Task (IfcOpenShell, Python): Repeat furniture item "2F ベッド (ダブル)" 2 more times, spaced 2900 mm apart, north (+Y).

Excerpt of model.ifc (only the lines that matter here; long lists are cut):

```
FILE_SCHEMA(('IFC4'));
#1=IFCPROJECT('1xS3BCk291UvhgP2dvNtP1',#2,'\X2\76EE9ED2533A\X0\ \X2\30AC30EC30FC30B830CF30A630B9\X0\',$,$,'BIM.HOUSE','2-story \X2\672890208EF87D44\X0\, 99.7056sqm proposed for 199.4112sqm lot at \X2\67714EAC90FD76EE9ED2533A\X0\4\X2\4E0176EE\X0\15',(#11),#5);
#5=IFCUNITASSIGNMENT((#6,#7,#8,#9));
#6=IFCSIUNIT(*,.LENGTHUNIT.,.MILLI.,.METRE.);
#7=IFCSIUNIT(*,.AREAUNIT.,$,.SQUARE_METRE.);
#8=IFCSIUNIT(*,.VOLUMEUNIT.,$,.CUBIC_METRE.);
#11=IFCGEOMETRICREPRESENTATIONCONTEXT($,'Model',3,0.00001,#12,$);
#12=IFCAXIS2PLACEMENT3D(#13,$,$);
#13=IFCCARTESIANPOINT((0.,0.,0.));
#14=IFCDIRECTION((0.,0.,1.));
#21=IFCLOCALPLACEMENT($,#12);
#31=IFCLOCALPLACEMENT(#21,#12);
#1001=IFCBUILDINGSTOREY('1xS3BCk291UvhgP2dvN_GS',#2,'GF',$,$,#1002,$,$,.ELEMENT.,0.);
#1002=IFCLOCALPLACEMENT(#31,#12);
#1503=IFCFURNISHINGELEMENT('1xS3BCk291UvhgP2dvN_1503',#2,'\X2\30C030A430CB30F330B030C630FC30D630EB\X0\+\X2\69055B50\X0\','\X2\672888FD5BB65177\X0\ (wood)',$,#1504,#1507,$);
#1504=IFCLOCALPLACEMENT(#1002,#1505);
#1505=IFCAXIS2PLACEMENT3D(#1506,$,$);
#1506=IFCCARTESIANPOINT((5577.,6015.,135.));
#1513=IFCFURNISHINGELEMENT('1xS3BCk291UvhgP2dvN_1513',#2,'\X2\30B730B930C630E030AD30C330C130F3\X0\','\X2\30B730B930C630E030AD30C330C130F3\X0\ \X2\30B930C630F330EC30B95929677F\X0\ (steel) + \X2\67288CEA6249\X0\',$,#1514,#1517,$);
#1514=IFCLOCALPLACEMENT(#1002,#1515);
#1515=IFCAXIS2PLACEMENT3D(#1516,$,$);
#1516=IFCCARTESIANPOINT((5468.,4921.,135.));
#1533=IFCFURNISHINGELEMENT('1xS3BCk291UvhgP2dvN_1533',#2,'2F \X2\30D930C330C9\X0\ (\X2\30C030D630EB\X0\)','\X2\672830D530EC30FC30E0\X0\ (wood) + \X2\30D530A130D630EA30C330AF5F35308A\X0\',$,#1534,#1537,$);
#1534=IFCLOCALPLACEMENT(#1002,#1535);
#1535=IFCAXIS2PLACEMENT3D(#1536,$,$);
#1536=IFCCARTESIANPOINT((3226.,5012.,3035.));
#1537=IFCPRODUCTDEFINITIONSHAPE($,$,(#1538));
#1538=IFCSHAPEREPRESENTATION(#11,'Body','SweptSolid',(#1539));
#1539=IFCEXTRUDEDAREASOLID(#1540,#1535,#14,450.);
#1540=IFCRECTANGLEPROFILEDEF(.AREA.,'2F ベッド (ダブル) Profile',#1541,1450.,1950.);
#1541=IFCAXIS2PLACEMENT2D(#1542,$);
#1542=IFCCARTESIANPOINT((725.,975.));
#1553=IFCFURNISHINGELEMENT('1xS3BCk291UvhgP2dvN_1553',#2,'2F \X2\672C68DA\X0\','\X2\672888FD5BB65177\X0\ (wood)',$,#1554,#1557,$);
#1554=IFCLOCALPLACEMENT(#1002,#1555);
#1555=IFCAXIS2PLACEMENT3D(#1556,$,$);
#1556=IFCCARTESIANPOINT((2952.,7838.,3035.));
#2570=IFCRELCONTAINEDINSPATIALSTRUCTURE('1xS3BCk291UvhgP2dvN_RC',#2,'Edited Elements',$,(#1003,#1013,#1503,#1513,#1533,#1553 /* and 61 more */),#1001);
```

```python
import numpy as np
import ifcopenshell
import ifcopenshell.api.geometry
import ifcopenshell.api.root
import ifcopenshell.util.element
import ifcopenshell.util.placement

model = ifcopenshell.open("model.ifc")


def reuse_history(source, copy):
    """copy_class also copies each property set's owner history, people and application; keep the originals."""
    for rel in copy.IsDefinedBy:
        if rel.is_a("IfcRelDefinesByProperties") and (history := rel.RelatingPropertyDefinition.OwnerHistory):
            rel.RelatingPropertyDefinition.OwnerHistory = source.OwnerHistory
            ifcopenshell.util.element.remove_deep2(model, history)


source = model.by_guid("1xS3BCk291UvhgP2dvN_1533")
base = ifcopenshell.util.placement.get_local_placement(source.ObjectPlacement)
step = np.array([0.0, 1.0, 0.0]) * 2900.0

for i in range(1, 3):
    copy = ifcopenshell.api.root.copy_class(model, product=source)
    copy.Representation = ifcopenshell.util.element.copy_deep(
        model, source.Representation, exclude=["IfcGeometricRepresentationContext", "IfcRepresentationMap"]
    )
    reuse_history(source, copy)
    matrix = base.copy()
    matrix[:3, 3] += i * step
    print("added at", matrix[:3, 3].round(3) + 0.0)
    ifcopenshell.api.geometry.edit_object_placement(model, product=copy, matrix=matrix, is_si=False)

model.write("model_v2.ifc")
```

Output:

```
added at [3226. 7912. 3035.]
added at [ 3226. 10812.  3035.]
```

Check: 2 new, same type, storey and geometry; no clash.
